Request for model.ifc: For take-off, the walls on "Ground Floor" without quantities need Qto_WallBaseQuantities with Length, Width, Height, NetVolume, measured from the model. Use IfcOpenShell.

First a look at what the model holds.

```python
import ifcopenshell
import ifcopenshell.util.element
import ifcopenshell.util.unit

model = ifcopenshell.open("model.ifc")
print(model.schema)
for unit_type in ("LENGTHUNIT", "AREAUNIT", "VOLUMEUNIT"):
    print(unit_type, ifcopenshell.util.unit.calculate_unit_scale(model, unit_type))
storey = next(s for s in model.by_type("IfcBuildingStorey") if s.Name == "Ground Floor")
walls = [e for e in ifcopenshell.util.element.get_decomposition(storey) if e.is_a("IfcWall")]
for e in sorted(walls, key=lambda e: e.id()):
    print(e.id(), e.is_a(), e.Name, list(ifcopenshell.util.element.get_psets(e, qtos_only=True)), sep=" | ")
```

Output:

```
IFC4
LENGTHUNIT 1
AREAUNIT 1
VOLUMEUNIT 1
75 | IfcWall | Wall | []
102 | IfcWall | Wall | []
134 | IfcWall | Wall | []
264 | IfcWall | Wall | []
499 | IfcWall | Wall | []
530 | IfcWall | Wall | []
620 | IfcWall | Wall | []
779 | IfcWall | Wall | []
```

```python
import ifcopenshell
import ifcopenshell.api.pset
import ifcopenshell.geom
import ifcopenshell.util.element
import ifcopenshell.util.shape
import ifcopenshell.util.unit

model = ifcopenshell.open("model.ifc")
unit_scale = ifcopenshell.util.unit.calculate_unit_scale(model)
volume_scale = ifcopenshell.util.unit.calculate_unit_scale(model, "VOLUMEUNIT")
settings = ifcopenshell.geom.settings()

storey = next(s for s in model.by_type("IfcBuildingStorey") if s.Name == "Ground Floor")
walls = [e for e in ifcopenshell.util.element.get_decomposition(storey) if e.is_a("IfcWall")]

for e in sorted(walls, key=lambda e: e.id()):
    if ifcopenshell.util.element.get_psets(e, qtos_only=True, should_inherit=False):
        continue
    # Geometry comes back in metres, in the element's own axes.
    shape = ifcopenshell.geom.create_shape(settings, e)
    values = {
        "Length": ifcopenshell.util.shape.get_x(shape.geometry) / unit_scale,
        "Width": ifcopenshell.util.shape.get_y(shape.geometry) / unit_scale,
        "Height": ifcopenshell.util.shape.get_z(shape.geometry) / unit_scale,
        "NetVolume": ifcopenshell.util.shape.get_volume(shape.geometry) / volume_scale,
    }
    qto = ifcopenshell.api.pset.add_qto(model, product=e, name="Qto_WallBaseQuantities")
    ifcopenshell.api.pset.edit_qto(model, qto=qto, properties=values)
    print(e.id(), {k: round(v, 3) for k, v in values.items()})

model.write("model_v2.ifc")
```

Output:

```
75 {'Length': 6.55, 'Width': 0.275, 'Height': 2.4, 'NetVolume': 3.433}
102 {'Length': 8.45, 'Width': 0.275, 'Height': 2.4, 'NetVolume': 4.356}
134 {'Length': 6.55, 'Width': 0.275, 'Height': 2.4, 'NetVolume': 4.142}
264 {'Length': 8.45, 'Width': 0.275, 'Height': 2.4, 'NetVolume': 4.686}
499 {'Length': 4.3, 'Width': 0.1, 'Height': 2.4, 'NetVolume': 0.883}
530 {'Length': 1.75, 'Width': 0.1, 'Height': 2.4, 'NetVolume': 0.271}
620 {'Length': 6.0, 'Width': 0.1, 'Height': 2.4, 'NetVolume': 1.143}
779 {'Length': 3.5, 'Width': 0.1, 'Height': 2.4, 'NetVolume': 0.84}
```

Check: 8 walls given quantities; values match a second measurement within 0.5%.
